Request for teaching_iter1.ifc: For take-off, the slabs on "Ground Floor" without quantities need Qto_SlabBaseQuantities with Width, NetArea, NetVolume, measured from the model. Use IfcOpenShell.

First a look at what the model holds.

```python
import ifcopenshell
import ifcopenshell.util.element
import ifcopenshell.util.unit

model = ifcopenshell.open("teaching_iter1.ifc")
print(model.schema)
for unit_type in ("LENGTHUNIT", "AREAUNIT", "VOLUMEUNIT"):
    print(unit_type, ifcopenshell.util.unit.calculate_unit_scale(model, unit_type))
storey = next(s for s in model.by_type("IfcBuildingStorey") if s.Name == "Ground Floor")
slabs = [e for e in ifcopenshell.util.element.get_decomposition(storey) if e.is_a("IfcSlab")]
for e in sorted(slabs, key=lambda e: e.id()):
    print(e.id(), e.is_a(), e.Name, list(ifcopenshell.util.element.get_psets(e, qtos_only=True)), sep=" | ")
```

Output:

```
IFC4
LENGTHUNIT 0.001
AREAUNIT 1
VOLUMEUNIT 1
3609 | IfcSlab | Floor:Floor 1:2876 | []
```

```python
import ifcopenshell
import ifcopenshell.api.pset
import ifcopenshell.geom
import ifcopenshell.util.element
import ifcopenshell.util.shape
import ifcopenshell.util.unit

model = ifcopenshell.open("teaching_iter1.ifc")
unit_scale = ifcopenshell.util.unit.calculate_unit_scale(model)
area_scale = ifcopenshell.util.unit.calculate_unit_scale(model, "AREAUNIT")
volume_scale = ifcopenshell.util.unit.calculate_unit_scale(model, "VOLUMEUNIT")
settings = ifcopenshell.geom.settings()

storey = next(s for s in model.by_type("IfcBuildingStorey") if s.Name == "Ground Floor")
slabs = [e for e in ifcopenshell.util.element.get_decomposition(storey) if e.is_a("IfcSlab")]

for e in sorted(slabs, key=lambda e: e.id()):
    if ifcopenshell.util.element.get_psets(e, qtos_only=True, should_inherit=False):
        continue
    # Geometry comes back in metres, in the element's own axes.
    shape = ifcopenshell.geom.create_shape(settings, e)
    values = {
        "Width": ifcopenshell.util.shape.get_z(shape.geometry) / unit_scale,
        "NetArea": ifcopenshell.util.shape.get_footprint_area(shape.geometry) / area_scale,
        "NetVolume": ifcopenshell.util.shape.get_volume(shape.geometry) / volume_scale,
    }
    qto = ifcopenshell.api.pset.add_qto(model, product=e, name="Qto_SlabBaseQuantities")
    ifcopenshell.api.pset.edit_qto(model, qto=qto, properties=values)
    print(e.id(), {k: round(v, 3) for k, v in values.items()})

model.write("teaching_iter1_v2.ifc")
```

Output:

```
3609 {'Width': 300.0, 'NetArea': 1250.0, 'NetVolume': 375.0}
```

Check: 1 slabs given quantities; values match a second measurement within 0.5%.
